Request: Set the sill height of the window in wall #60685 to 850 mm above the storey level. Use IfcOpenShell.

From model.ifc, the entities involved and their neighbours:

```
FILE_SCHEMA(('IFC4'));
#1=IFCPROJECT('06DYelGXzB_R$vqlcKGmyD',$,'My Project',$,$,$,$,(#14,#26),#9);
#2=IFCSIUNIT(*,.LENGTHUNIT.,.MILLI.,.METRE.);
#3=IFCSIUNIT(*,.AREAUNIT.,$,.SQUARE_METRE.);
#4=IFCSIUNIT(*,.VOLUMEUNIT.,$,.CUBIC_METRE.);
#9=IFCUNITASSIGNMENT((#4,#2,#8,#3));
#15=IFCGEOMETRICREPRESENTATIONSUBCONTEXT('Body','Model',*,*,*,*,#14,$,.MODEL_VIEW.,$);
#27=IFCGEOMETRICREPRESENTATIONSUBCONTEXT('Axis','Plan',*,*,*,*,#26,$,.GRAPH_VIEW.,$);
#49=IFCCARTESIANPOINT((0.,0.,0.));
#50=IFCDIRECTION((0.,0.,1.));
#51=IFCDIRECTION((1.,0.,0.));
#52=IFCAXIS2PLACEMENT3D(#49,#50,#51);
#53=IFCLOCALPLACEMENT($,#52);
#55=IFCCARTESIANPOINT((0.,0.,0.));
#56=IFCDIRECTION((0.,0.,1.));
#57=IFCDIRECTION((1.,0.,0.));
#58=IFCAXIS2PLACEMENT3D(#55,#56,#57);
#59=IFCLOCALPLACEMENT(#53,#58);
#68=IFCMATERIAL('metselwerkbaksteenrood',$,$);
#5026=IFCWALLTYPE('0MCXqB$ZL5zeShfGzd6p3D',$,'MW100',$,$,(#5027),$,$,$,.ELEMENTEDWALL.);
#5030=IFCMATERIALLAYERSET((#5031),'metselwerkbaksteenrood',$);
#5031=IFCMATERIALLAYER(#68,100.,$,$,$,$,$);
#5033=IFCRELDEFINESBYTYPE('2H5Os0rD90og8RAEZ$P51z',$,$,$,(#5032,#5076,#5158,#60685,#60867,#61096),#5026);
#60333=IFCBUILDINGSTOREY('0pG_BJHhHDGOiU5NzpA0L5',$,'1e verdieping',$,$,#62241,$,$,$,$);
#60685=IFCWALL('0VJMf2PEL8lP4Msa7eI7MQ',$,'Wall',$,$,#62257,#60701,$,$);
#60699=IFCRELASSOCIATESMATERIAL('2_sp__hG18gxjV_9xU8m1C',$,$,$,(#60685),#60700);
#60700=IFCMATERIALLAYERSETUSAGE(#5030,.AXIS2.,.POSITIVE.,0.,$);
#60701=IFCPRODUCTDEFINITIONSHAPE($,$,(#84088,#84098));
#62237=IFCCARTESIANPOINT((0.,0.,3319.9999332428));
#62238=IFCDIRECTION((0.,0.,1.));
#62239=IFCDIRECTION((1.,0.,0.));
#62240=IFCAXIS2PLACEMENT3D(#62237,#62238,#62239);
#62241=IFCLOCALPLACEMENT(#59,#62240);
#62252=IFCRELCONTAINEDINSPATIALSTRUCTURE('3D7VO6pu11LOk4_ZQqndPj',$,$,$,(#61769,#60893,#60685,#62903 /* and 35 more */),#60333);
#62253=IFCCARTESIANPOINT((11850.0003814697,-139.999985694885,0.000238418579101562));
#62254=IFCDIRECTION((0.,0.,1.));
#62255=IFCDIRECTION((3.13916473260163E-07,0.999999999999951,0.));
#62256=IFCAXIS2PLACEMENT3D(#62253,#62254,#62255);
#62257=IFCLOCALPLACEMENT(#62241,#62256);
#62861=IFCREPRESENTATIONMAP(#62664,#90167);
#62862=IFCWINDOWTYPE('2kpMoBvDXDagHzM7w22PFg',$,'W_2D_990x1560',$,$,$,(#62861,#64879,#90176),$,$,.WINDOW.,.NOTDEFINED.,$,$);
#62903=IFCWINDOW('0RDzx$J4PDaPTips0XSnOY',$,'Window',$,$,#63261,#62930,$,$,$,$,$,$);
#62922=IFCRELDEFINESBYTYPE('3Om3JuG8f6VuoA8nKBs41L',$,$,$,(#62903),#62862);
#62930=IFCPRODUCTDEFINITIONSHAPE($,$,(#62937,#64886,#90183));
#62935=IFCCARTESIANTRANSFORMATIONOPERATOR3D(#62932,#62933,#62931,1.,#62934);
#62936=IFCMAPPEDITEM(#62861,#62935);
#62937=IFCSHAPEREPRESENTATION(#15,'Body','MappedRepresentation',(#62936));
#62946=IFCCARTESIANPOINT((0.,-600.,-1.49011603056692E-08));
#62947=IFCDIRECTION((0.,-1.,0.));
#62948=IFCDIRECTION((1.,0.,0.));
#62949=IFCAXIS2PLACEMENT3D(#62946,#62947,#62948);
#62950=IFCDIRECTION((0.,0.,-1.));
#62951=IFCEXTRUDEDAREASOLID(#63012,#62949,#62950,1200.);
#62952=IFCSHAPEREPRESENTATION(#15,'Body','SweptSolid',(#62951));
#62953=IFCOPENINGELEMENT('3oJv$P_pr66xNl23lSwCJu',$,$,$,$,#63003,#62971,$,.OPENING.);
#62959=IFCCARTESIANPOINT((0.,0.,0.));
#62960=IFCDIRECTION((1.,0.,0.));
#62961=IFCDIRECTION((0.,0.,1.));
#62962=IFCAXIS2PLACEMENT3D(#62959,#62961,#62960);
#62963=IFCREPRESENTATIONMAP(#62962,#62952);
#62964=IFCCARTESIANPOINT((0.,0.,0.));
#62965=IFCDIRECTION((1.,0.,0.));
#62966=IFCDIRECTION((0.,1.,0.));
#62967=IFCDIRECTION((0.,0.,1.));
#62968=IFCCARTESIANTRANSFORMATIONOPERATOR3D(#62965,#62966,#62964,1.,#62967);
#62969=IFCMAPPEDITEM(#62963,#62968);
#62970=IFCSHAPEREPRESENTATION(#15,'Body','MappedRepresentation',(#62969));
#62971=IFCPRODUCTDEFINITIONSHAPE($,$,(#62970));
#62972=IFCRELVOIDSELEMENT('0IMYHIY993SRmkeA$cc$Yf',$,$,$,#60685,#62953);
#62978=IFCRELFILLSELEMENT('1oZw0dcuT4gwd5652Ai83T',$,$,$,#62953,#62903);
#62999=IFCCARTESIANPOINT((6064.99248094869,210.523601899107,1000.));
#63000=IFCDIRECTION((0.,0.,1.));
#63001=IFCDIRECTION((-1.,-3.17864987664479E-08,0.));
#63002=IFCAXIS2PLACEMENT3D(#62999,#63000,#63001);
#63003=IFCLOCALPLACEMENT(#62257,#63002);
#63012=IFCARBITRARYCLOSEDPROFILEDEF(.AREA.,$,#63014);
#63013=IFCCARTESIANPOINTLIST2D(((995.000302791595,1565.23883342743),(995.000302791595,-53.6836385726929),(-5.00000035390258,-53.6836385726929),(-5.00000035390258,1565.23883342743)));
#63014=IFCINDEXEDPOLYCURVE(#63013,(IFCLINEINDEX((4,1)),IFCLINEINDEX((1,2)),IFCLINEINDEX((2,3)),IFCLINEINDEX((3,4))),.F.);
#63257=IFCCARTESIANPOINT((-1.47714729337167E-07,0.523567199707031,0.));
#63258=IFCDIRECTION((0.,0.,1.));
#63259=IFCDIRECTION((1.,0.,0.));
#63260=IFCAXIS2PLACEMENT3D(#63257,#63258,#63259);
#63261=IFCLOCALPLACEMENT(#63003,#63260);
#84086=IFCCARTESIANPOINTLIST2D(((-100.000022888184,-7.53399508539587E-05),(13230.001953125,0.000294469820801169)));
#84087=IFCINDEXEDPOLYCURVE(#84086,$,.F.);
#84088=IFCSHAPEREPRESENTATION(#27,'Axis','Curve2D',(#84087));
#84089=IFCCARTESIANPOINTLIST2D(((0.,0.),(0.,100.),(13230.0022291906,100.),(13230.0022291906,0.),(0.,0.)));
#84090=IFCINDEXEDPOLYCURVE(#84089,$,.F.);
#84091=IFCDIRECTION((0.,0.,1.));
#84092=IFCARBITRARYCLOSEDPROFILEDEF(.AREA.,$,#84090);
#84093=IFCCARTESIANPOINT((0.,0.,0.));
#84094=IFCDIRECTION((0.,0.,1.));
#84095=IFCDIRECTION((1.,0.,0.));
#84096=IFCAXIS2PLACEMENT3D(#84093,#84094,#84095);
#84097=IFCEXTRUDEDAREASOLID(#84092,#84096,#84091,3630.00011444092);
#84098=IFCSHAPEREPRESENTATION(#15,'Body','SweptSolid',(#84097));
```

```python
import numpy as np
import ifcopenshell
import ifcopenshell.api.geometry
import ifcopenshell.geom
import ifcopenshell.util.element
import ifcopenshell.util.placement
import ifcopenshell.util.shape
import ifcopenshell.util.unit

model = ifcopenshell.open("model.ifc")
unit_scale = ifcopenshell.util.unit.calculate_unit_scale(model)

window = model.by_guid("0RDzx$J4PDaPTips0XSnOY")
opening = window.FillsVoids[0].RelatingOpeningElement
storey = ifcopenshell.util.element.get_container(window, ifc_class="IfcBuildingStorey")
level = ifcopenshell.util.placement.get_local_placement(storey.ObjectPlacement)[2, 3]

# The opening's origin need not be at the sill, so measure its lowest point.
shape = ifcopenshell.geom.create_shape(ifcopenshell.geom.settings(), opening)
bottom = ifcopenshell.util.shape.get_shape_bottom_elevation(shape, shape.geometry) / unit_scale
dz = level + 0.85 / unit_scale - bottom

shift = np.array([0.0, 0.0, dz])
# The window is placed relative to its opening, so it follows when the opening moves.
matrix = ifcopenshell.util.placement.get_local_placement(opening.ObjectPlacement)
matrix[:3, 3] += shift
ifcopenshell.api.geometry.edit_object_placement(
    model, product=opening, matrix=matrix, is_si=False, should_transform_children=True
)

print(f"moved by {dz * unit_scale:+.3f} m")

model.write("model_rev.ifc")
```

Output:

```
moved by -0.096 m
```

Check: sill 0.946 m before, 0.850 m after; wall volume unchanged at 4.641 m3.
